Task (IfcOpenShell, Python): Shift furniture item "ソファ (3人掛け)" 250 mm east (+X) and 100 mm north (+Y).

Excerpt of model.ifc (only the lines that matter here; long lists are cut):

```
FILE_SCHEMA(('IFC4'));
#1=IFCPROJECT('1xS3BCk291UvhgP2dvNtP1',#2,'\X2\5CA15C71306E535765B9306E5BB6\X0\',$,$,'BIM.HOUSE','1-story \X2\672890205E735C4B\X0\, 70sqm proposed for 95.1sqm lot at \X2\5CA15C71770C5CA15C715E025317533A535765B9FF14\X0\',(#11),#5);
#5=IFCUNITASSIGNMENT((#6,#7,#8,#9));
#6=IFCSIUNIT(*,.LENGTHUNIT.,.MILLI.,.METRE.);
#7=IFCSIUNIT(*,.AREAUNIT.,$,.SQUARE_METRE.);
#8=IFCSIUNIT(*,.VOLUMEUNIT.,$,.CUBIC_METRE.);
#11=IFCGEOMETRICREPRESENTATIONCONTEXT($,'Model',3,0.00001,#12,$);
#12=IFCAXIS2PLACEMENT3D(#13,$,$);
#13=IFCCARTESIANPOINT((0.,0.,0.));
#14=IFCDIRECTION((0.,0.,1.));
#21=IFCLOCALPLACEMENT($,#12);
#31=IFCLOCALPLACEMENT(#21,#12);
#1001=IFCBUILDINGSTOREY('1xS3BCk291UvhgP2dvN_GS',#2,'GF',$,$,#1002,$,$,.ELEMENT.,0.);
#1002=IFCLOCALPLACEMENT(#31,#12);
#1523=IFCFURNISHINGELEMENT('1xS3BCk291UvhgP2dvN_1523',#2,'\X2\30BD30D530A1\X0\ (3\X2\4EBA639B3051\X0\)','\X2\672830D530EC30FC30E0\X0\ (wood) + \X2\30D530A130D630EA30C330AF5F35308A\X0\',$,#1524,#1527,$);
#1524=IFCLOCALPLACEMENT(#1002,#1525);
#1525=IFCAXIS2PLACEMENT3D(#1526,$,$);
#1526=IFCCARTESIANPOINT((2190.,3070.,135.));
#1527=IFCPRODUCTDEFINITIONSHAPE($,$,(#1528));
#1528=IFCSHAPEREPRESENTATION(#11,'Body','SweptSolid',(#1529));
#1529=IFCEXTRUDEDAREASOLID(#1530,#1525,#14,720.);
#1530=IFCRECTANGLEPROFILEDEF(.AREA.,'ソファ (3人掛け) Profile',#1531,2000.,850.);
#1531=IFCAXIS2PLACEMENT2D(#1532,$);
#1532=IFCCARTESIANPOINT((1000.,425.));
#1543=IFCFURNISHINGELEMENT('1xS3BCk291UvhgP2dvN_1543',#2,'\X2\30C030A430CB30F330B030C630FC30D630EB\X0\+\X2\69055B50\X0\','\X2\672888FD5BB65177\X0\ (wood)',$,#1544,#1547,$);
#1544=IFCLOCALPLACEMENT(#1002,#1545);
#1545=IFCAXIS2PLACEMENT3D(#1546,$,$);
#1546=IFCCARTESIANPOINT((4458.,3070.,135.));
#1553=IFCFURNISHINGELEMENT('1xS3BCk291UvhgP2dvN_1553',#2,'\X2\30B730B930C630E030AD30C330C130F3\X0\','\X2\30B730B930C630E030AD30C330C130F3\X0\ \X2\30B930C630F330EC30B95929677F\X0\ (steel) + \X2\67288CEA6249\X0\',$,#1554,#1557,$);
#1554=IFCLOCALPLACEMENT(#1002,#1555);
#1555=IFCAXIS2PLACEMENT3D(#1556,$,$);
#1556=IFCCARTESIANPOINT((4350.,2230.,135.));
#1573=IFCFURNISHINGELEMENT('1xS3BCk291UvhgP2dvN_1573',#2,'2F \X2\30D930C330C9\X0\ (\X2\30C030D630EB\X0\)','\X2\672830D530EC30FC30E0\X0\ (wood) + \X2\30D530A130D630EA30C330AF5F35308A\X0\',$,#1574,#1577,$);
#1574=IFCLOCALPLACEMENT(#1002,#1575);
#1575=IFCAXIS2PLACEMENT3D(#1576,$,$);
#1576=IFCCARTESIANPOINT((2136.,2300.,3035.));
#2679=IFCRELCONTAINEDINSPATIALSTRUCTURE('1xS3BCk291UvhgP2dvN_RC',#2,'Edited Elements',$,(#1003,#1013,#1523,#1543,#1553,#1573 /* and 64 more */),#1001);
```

```python
import ifcopenshell
import ifcopenshell.api.geometry
import ifcopenshell.util.placement
import ifcopenshell.util.unit

model = ifcopenshell.open("model.ifc")
unit_scale = ifcopenshell.util.unit.calculate_unit_scale(model)

item = model.by_id(1523)
matrix = ifcopenshell.util.placement.get_local_placement(item.ObjectPlacement)
matrix[0, 3] += 0.25 / unit_scale
matrix[1, 3] += 0.1 / unit_scale
ifcopenshell.api.geometry.edit_object_placement(model, product=item, matrix=matrix, is_si=False)

print(ifcopenshell.util.placement.get_local_placement(item.ObjectPlacement).round(3) + 0.0)

model.write("model-out.ifc")
```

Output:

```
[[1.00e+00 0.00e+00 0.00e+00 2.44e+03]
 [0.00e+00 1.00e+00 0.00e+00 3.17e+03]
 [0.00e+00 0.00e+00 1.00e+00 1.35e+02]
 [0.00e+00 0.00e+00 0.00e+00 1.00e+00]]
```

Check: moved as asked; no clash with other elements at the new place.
